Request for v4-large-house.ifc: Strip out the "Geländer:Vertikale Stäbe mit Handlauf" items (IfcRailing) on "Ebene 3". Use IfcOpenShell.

First a look at what the model holds.

```python
import ifcopenshell
import ifcopenshell.util.element

model = ifcopenshell.open("v4-large-house.ifc")
print(model.schema)
storey = next(s for s in model.by_type("IfcBuildingStorey") if s.Name == "Ebene 3")
railings = [e for e in ifcopenshell.util.element.get_decomposition(storey) if e.is_a("IfcRailing")]
seen = {}
for e in railings:
    element_type = ifcopenshell.util.element.get_type(e)
    name = element_type.Name if element_type not in (None, e) else None
    seen[name] = seen.get(name, 0) + 1
for name, count in sorted(seen.items(), key=str):
    print(count, "x", name)
```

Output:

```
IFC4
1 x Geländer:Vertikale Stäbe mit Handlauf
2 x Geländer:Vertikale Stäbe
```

```python
import ifcopenshell
import ifcopenshell.api.root
import ifcopenshell.util.element

model = ifcopenshell.open("v4-large-house.ifc")

storey = next(s for s in model.by_type("IfcBuildingStorey") if s.Name == "Ebene 3")
railings = [e for e in ifcopenshell.util.element.get_decomposition(storey) if e.is_a("IfcRailing")]
targets = [e for e in railings if (t := ifcopenshell.util.element.get_type(e)) not in (None, e) and t.Name == "Geländer:Vertikale Stäbe mit Handlauf"]

for e in targets:
    ifcopenshell.api.root.remove_product(model, product=e)
print(len(targets), "removed")

model.write("v4-large-house-out.ifc")
```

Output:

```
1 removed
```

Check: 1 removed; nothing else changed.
